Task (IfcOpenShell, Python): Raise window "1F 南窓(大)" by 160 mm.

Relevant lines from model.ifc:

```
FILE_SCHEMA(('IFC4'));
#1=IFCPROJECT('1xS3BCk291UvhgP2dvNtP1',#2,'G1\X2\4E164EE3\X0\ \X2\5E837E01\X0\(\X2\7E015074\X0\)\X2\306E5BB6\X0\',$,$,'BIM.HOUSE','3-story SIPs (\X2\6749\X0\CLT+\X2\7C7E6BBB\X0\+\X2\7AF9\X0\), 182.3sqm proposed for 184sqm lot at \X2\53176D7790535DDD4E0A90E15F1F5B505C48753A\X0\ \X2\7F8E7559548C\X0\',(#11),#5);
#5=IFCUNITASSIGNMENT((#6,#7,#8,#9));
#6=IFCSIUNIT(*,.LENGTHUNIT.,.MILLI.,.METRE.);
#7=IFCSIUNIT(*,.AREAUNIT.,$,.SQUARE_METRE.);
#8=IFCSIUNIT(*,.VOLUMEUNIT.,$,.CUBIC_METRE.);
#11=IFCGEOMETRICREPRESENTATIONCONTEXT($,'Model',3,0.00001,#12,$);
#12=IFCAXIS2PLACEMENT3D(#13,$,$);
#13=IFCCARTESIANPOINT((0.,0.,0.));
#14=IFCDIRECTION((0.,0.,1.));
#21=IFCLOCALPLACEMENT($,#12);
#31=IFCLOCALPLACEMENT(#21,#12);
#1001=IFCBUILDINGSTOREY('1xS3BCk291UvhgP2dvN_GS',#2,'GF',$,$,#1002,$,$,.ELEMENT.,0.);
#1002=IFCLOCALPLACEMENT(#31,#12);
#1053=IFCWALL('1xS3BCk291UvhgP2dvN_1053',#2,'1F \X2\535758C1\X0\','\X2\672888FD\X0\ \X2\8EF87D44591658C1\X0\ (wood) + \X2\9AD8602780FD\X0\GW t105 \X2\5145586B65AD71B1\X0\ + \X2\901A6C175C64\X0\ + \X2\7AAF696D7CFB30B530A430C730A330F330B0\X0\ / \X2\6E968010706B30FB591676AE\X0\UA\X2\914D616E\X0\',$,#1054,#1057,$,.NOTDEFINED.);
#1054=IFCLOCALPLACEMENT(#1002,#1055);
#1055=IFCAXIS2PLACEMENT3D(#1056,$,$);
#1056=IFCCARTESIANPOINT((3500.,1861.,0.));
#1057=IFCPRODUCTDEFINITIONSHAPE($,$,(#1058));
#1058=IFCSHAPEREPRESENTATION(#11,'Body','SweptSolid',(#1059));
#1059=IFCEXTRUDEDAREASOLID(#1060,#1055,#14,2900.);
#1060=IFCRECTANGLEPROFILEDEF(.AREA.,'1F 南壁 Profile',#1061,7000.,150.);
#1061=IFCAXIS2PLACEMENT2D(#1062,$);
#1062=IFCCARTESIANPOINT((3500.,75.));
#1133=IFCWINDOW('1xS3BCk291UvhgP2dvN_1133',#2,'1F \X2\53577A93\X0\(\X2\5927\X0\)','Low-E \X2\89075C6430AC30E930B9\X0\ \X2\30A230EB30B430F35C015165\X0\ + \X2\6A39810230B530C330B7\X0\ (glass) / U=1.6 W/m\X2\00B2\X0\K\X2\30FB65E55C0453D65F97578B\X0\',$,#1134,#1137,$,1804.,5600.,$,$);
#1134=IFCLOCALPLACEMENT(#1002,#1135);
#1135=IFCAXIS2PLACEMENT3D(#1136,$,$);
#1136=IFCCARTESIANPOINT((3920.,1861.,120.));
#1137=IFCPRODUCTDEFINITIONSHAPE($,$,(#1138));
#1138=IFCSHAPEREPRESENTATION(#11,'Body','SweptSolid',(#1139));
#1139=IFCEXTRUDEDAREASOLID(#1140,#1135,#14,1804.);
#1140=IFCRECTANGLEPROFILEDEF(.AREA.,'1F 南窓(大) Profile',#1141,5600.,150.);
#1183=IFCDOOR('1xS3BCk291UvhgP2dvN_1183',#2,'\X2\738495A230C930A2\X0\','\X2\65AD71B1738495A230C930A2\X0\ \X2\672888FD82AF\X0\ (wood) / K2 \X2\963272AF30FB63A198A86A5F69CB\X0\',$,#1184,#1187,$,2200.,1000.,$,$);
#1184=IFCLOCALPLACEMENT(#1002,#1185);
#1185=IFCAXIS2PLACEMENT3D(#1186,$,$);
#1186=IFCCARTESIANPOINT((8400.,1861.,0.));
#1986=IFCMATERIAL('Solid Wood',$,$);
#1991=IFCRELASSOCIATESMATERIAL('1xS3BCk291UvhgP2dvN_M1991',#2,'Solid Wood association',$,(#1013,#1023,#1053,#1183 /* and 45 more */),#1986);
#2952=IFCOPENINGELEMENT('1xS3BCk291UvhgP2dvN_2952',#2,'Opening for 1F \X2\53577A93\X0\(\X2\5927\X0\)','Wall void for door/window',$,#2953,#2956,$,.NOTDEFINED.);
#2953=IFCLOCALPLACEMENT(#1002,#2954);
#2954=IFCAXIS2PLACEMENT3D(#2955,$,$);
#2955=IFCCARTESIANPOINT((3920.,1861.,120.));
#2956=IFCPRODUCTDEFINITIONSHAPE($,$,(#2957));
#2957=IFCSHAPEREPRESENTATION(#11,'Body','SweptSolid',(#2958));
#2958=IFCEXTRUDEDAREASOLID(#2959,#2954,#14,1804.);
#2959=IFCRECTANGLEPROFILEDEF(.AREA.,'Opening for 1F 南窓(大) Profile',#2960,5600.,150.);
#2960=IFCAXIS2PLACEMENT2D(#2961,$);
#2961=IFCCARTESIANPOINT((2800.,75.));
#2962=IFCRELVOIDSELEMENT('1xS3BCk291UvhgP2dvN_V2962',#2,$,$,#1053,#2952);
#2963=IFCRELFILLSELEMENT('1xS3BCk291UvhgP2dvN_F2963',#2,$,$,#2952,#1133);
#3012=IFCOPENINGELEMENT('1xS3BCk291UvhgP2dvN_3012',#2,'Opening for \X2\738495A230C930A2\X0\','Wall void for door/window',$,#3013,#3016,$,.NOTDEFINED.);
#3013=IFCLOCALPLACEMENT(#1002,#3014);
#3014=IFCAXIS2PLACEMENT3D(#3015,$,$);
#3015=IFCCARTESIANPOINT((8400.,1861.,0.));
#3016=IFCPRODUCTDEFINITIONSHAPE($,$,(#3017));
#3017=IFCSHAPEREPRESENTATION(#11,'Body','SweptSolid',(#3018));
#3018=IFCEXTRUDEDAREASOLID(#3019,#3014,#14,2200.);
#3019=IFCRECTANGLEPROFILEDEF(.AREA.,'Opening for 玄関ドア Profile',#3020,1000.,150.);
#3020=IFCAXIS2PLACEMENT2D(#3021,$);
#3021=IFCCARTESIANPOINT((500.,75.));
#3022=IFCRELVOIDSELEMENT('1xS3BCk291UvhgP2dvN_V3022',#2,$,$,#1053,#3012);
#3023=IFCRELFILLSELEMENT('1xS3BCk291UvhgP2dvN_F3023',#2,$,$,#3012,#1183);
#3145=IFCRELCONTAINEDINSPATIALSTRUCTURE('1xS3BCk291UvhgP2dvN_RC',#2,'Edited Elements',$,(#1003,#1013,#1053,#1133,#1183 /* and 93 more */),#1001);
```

```python
import numpy as np
import ifcopenshell
import ifcopenshell.api.geometry
import ifcopenshell.util.placement
import ifcopenshell.util.unit

model = ifcopenshell.open("model.ifc")
unit_scale = ifcopenshell.util.unit.calculate_unit_scale(model)

window = model.by_guid("1xS3BCk291UvhgP2dvN_1133")
opening = window.FillsVoids[0].RelatingOpeningElement
dz = 0.16 / unit_scale

shift = np.array([0.0, 0.0, dz])
# The window is not placed relative to its opening, so move both.
for product in (opening, window):
    matrix = ifcopenshell.util.placement.get_local_placement(product.ObjectPlacement)
    matrix[:3, 3] += shift
    ifcopenshell.api.geometry.edit_object_placement(model, product=product, matrix=matrix, is_si=False)

print(f"moved by {dz * unit_scale:+.3f} m")

model.write("model-out.ifc")
```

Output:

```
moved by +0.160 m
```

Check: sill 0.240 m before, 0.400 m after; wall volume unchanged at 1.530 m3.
